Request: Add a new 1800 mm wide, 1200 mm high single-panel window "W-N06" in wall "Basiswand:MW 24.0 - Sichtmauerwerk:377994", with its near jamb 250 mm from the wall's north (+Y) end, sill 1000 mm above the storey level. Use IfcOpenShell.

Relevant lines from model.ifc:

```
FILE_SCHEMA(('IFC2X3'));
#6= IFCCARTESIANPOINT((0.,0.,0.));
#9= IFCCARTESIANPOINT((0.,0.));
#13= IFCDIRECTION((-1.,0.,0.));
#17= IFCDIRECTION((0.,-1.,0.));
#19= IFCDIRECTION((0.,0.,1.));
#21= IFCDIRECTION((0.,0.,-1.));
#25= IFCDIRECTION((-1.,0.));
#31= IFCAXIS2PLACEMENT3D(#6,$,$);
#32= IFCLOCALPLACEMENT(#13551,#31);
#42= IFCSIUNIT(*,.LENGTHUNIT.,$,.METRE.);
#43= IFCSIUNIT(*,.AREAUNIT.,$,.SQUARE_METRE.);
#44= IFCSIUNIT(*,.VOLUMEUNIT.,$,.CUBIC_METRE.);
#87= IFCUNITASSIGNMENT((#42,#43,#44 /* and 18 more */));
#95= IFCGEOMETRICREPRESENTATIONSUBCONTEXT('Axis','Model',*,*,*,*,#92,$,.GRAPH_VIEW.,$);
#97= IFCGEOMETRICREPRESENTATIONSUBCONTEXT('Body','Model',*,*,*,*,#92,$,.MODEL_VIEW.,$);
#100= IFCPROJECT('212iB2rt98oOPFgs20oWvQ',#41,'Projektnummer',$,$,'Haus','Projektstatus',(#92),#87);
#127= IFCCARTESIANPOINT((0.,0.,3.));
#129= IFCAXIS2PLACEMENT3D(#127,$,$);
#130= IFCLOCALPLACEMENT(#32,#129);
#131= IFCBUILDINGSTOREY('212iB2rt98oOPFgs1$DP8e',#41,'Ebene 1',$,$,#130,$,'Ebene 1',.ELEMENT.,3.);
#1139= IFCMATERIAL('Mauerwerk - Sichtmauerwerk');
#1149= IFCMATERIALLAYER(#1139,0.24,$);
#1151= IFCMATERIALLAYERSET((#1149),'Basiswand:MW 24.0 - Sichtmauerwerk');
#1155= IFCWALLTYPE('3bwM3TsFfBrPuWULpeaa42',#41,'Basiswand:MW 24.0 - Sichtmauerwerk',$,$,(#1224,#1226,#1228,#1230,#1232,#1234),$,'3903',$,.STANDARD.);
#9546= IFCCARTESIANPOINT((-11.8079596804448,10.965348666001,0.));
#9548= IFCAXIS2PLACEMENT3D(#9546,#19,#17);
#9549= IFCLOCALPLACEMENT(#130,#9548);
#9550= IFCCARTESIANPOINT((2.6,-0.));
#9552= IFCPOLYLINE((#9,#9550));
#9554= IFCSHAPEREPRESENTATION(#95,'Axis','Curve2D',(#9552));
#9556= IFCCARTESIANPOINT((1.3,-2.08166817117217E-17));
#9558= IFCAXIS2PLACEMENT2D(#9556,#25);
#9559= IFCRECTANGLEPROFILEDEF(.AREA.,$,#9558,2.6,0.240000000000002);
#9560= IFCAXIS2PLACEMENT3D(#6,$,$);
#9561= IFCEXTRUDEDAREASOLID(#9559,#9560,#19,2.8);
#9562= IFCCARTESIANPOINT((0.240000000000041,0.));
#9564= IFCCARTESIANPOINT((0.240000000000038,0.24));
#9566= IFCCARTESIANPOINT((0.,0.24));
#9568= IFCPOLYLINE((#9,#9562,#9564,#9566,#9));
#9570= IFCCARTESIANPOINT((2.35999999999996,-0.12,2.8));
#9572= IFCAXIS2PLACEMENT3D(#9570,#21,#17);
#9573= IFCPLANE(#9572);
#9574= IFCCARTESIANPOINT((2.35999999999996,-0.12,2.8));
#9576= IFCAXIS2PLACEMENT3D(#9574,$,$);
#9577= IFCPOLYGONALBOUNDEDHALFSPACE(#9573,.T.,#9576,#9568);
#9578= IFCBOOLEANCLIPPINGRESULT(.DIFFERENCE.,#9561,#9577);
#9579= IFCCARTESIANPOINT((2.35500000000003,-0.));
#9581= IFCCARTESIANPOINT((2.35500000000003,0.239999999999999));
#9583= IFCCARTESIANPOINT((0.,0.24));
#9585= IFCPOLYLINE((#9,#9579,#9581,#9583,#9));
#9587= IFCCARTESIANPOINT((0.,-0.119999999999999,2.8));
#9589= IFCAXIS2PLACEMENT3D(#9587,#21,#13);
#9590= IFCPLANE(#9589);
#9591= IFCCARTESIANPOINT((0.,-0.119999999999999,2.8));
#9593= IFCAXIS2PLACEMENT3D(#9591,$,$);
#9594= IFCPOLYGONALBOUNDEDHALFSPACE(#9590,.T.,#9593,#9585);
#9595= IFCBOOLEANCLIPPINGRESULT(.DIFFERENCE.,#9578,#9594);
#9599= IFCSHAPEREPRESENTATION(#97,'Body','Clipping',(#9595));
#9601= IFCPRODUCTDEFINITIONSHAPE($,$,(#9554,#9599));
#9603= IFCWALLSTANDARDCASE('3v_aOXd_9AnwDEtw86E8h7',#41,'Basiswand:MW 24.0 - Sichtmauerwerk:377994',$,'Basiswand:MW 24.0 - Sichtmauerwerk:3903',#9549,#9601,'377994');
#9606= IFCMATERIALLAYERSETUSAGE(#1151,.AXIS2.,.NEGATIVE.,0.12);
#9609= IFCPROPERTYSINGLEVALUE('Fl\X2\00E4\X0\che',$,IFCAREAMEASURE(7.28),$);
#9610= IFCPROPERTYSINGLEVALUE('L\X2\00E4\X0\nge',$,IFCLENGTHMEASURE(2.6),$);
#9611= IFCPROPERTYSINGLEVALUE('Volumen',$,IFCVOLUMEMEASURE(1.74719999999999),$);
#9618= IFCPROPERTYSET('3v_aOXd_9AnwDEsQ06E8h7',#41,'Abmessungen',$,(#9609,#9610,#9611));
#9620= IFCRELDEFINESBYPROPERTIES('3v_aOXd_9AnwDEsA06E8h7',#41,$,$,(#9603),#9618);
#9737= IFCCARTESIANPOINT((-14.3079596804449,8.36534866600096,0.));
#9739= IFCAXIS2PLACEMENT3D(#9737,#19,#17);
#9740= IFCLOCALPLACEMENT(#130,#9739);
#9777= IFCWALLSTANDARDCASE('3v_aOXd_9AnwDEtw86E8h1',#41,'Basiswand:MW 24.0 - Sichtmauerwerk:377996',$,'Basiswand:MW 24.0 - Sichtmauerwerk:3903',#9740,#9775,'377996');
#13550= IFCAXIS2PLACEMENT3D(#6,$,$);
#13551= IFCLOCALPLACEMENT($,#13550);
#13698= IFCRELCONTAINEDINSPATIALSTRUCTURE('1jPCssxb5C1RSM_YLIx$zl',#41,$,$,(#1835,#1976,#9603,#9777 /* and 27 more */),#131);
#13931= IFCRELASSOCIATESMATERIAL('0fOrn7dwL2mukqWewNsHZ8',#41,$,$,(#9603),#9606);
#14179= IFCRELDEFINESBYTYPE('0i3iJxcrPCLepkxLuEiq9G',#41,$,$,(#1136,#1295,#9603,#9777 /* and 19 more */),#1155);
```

```python
import numpy as np
import ifcopenshell
import ifcopenshell.api.feature
import ifcopenshell.api.geometry
import ifcopenshell.api.pset
import ifcopenshell.api.root
import ifcopenshell.api.spatial
import ifcopenshell.api.type
import ifcopenshell.geom
import ifcopenshell.util.element
import ifcopenshell.util.placement
import ifcopenshell.util.representation
import ifcopenshell.util.shape
import ifcopenshell.util.unit

model = ifcopenshell.open("model.ifc")
unit_scale = ifcopenshell.util.unit.calculate_unit_scale(model)
area_scale = ifcopenshell.util.unit.calculate_unit_scale(model, "AREAUNIT")
volume_scale = ifcopenshell.util.unit.calculate_unit_scale(model, "VOLUMEUNIT")
settings = ifcopenshell.geom.settings()


def volume(element):
    """Net volume in cubic metres, openings subtracted."""
    shape = ifcopenshell.geom.create_shape(settings, element)
    return ifcopenshell.util.shape.get_volume(shape.geometry)


wall = model.by_id(9603)
storey = ifcopenshell.util.element.get_container(wall, ifc_class="IfcBuildingStorey")
context = ifcopenshell.util.representation.get_context(model, "Model", "Body", "MODEL_VIEW")
before = volume(wall)

width, height, from_end, sill = 1.8, 1.2, 0.25, 1  # metres

# The wall runs along its own X axis, and the end named is its -X end.
wall_shape = ifcopenshell.geom.create_shape(settings, wall)
x, y, z = ifcopenshell.util.shape.get_vertices(wall_shape.geometry).T
start = x.min() + from_end
face, thickness = float(y.min()), float(y.max() - y.min())
wall_matrix = ifcopenshell.util.placement.get_local_placement(wall.ObjectPlacement)
level = ifcopenshell.util.placement.get_local_placement(storey.ObjectPlacement)[2, 3]


def in_wall(x, y):
    """Placement at x, y metres in the wall's axes, at sill height."""
    matrix = wall_matrix.copy()
    matrix[:, 3] = wall_matrix @ np.array([x / unit_scale, y / unit_scale, 0.0, 1.0])
    matrix[2, 3] = level + sill / unit_scale
    return matrix


# Opening: a box that overshoots both wall faces by 50 mm.
opening = ifcopenshell.api.root.create_entity(model, ifc_class="IfcOpeningElement")
box = ifcopenshell.api.geometry.add_wall_representation(
    model, context=context, length=width, height=height, thickness=thickness + 0.1
)
ifcopenshell.api.geometry.assign_representation(model, product=opening, representation=box)
ifcopenshell.api.geometry.edit_object_placement(model, product=opening, matrix=in_wall(start, face - 0.05), is_si=False)
ifcopenshell.api.feature.add_feature(model, feature=opening, element=wall)

window = ifcopenshell.api.root.create_entity(model, ifc_class="IfcWindow", name="W-N06")
window.OverallWidth, window.OverallHeight = width / unit_scale, height / unit_scale
body = ifcopenshell.api.geometry.add_window_representation(
    model,
    context=context,
    overall_width=window.OverallWidth,
    overall_height=window.OverallHeight,
    partition_type="SINGLE_PANEL",
)
ifcopenshell.api.geometry.assign_representation(model, product=window, representation=body)
ifcopenshell.api.spatial.assign_container(model, products=[window], relating_structure=storey)
fills = ifcopenshell.api.feature.add_filling(model, opening=opening, element=window)
fills.OwnerHistory = window.OwnerHistory  # required in IFC2X3

# IFC2X3 keeps the operation on the window style.
style = ifcopenshell.api.root.create_entity(model, ifc_class="IfcWindowStyle", name="W-N06")
style.OperationType, style.ConstructionType = "SINGLE_PANEL", "NOTDEFINED"
style.ParameterTakesPrecedence = style.Sizeable = False
ifcopenshell.api.type.assign_type(model, related_objects=[window], relating_type=style)

# Centre the window in the wall's thickness.
ifcopenshell.api.geometry.edit_object_placement(model, product=window, matrix=in_wall(start, face), is_si=False)
window_shape = ifcopenshell.geom.create_shape(settings, window)
depth = ifcopenshell.util.shape.get_vertices(window_shape.geometry)[:, 1]
offset = face + thickness / 2 - (depth.min() + depth.max()) / 2
ifcopenshell.api.geometry.edit_object_placement(model, product=window, matrix=in_wall(start, offset), is_si=False)

after = volume(wall)

# Update the wall's stored quantities.
pset = model.by_id(ifcopenshell.util.element.get_pset(wall, "Abmessungen", should_inherit=False)["id"])
ifcopenshell.api.pset.edit_pset(model, pset=pset, properties={
    "Fläche": model.create_entity("IfcAreaMeasure", after / thickness / area_scale),
    "Volumen": model.create_entity("IfcVolumeMeasure", after / volume_scale),
})

print(f"wall volume {before:.3f} -> {after:.3f} m3")

model.write("model_rev.ifc")
```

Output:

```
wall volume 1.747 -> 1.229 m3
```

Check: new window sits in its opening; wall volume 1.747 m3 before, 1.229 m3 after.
